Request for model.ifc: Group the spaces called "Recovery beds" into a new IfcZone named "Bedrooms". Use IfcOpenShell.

First a look at what the model holds.

```python
import ifcopenshell

model = ifcopenshell.open("model.ifc")
print(model.schema)
seen = {}
for space in model.by_type("IfcSpace"):
    seen[space.Name] = seen.get(space.Name, 0) + 1
for name, count in sorted(seen.items(), key=str):
    print(count, "x", name)
print("zones:", [z.Name for z in model.by_type("IfcZone")][:20])
```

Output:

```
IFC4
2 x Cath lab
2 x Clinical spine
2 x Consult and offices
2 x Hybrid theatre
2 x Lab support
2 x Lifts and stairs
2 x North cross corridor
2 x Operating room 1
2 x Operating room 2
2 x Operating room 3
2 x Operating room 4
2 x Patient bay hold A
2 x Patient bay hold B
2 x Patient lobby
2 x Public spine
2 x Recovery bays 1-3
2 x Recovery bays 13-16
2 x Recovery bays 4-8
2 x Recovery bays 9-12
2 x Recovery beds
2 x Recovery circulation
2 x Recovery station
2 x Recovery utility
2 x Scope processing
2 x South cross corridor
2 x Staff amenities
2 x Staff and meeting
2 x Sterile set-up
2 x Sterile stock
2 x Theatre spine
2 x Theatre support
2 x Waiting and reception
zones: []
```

```python
import ifcopenshell
import ifcopenshell.api.group
import ifcopenshell.api.root

model = ifcopenshell.open("model.ifc")

names = {"Recovery beds"}
spaces = [s for s in model.by_type("IfcSpace") if s.Name in names]

zone = ifcopenshell.api.root.create_entity(model, ifc_class="IfcZone", name="Bedrooms")
ifcopenshell.api.group.assign_group(model, products=spaces, group=zone)
print(len(spaces), "spaces in", zone.Name)

model.write("model_rev.ifc")
```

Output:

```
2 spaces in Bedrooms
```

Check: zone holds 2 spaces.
